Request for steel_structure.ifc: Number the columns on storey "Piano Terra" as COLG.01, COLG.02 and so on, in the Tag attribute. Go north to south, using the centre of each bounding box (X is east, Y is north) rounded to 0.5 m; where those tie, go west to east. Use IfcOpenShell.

First a look at what the model holds.

```python
import ifcopenshell
import ifcopenshell.util.element
import ifcopenshell.util.placement

model = ifcopenshell.open("steel_structure.ifc")
print(model.schema)
storey = next(s for s in model.by_type("IfcBuildingStorey") if s.Name == "Piano Terra")
columns = [e for e in ifcopenshell.util.element.get_decomposition(storey) if e.is_a("IfcColumn")]
for e in sorted(columns, key=lambda e: e.id()):
    origin = ifcopenshell.util.placement.get_local_placement(e.ObjectPlacement)[:3, 3]
    print(e.id(), e.Tag, e.Name, origin.round(2) + 0.0, sep=" | ")
```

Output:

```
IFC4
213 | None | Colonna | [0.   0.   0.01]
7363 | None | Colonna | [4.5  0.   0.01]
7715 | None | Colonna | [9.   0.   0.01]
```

```python
import ifcopenshell
import ifcopenshell.geom
import ifcopenshell.util.element
import ifcopenshell.util.shape

model = ifcopenshell.open("steel_structure.ifc")
settings = ifcopenshell.geom.settings()
settings.set("use-world-coords", True)


def centre(element):
    shape = ifcopenshell.geom.create_shape(settings, element)
    return ifcopenshell.util.shape.get_bbox_centroid(shape.geometry)


storey = next(s for s in model.by_type("IfcBuildingStorey") if s.Name == "Piano Terra")
columns = [e for e in ifcopenshell.util.element.get_decomposition(storey) if e.is_a("IfcColumn")]

# Insertion points can sit at a corner or the storey origin, so sort by the geometry (in metres).
centres = {e: centre(e) for e in columns}
columns.sort(key=lambda e: (-round(centres[e][1] / 0.5), centres[e][0]))

for i, e in enumerate(columns, start=1):
    number = f"COLG.{i:02d}"
    e.Tag = number
    print(e.id(), number)

model.write("steel_structure_edited.ifc")
```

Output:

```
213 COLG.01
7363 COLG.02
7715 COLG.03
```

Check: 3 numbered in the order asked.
